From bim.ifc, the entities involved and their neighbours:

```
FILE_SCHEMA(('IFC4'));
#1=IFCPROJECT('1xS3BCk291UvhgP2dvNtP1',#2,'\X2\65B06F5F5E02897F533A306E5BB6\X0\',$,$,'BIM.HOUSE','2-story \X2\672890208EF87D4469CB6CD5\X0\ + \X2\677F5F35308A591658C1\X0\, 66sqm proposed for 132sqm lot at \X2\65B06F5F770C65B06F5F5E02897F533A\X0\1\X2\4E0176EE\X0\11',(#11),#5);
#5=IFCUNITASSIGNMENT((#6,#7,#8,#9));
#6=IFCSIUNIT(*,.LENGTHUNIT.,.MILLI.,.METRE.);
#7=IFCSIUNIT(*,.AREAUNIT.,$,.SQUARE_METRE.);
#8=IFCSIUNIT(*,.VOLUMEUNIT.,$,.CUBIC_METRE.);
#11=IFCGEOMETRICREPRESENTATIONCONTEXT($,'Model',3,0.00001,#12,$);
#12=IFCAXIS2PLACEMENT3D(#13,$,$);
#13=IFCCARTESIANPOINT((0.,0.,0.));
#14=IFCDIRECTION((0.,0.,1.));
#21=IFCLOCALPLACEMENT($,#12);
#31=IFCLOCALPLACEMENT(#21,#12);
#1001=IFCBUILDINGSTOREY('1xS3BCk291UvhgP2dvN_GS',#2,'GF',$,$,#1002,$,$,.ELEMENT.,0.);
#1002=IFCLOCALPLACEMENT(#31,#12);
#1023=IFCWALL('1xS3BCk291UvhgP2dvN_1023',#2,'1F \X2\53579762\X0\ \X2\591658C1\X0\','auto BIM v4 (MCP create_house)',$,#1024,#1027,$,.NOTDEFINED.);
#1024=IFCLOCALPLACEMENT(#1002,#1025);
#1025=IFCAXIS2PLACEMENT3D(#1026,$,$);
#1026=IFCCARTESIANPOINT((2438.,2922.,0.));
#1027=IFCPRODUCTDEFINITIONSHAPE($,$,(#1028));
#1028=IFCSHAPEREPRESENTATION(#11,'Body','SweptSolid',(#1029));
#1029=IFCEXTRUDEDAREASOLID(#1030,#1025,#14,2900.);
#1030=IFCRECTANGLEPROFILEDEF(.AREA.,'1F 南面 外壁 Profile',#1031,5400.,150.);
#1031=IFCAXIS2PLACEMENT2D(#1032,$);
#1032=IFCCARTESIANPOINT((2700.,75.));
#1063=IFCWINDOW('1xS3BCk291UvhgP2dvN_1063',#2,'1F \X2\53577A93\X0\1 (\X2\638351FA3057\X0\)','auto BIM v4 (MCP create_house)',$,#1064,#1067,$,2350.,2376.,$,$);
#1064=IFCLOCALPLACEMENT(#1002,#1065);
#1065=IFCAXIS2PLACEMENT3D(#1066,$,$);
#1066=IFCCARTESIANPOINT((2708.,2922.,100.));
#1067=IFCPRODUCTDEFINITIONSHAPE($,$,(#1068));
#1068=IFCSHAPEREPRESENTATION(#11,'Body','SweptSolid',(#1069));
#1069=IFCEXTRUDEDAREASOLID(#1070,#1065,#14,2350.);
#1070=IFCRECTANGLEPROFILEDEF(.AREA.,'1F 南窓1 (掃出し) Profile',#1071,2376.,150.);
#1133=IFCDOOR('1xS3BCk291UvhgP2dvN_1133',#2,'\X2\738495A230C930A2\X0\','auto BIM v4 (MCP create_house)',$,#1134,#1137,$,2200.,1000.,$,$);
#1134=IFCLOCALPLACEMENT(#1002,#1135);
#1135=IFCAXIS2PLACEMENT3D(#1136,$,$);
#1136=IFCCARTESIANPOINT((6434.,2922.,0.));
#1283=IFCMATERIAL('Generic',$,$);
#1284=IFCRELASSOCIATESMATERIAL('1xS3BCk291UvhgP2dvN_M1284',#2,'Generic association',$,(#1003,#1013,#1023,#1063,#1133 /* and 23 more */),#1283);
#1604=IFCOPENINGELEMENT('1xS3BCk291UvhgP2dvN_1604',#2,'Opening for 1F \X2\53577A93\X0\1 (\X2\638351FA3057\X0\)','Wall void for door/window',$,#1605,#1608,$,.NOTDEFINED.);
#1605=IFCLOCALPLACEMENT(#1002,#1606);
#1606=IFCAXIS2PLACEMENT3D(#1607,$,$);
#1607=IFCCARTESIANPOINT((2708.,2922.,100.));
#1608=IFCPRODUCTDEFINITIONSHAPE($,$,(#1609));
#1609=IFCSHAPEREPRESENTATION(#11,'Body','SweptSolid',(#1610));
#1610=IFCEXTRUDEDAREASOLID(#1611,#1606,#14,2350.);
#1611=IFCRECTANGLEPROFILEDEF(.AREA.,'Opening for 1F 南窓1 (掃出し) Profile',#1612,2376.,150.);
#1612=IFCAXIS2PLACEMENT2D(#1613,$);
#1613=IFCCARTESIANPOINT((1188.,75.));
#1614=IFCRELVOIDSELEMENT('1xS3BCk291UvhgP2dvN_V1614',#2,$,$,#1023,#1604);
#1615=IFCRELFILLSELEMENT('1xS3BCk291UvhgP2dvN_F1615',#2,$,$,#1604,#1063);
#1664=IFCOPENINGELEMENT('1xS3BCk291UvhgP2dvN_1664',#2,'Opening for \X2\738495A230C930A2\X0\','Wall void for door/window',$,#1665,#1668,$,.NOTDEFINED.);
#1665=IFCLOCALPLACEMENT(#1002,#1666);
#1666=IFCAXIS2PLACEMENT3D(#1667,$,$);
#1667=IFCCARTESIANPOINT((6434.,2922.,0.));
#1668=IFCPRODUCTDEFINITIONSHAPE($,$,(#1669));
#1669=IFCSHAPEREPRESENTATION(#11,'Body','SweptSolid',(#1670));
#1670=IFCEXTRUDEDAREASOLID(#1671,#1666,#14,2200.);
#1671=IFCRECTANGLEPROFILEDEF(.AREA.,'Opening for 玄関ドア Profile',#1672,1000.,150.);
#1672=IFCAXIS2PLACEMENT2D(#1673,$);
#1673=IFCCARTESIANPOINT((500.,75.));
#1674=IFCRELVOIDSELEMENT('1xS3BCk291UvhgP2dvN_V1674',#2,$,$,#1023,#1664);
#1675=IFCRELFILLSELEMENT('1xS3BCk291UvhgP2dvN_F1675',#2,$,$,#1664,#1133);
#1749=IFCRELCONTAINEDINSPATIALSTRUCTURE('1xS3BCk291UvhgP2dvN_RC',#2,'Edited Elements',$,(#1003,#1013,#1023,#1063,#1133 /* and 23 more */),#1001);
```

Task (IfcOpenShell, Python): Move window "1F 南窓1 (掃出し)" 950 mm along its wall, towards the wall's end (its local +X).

```python
import ifcopenshell
import ifcopenshell.api.geometry
import ifcopenshell.util.placement
import ifcopenshell.util.unit

model = ifcopenshell.open("bim.ifc")
unit_scale = ifcopenshell.util.unit.calculate_unit_scale(model)

window = model.by_guid("1xS3BCk291UvhgP2dvN_1063")
opening = window.FillsVoids[0].RelatingOpeningElement
wall = opening.VoidsElements[0].RelatingBuildingElement

wall_matrix = ifcopenshell.util.placement.get_local_placement(wall.ObjectPlacement)
shift = wall_matrix[:3, 0] * 0.95 / unit_scale
before = ifcopenshell.util.placement.get_local_placement(window.ObjectPlacement)[:3, 3].copy()

# The window is not placed relative to its opening, so move both.
for product in (opening, window):
    matrix = ifcopenshell.util.placement.get_local_placement(product.ObjectPlacement)
    matrix[:3, 3] += shift
    ifcopenshell.api.geometry.edit_object_placement(model, product=product, matrix=matrix, is_si=False)

after = ifcopenshell.util.placement.get_local_placement(window.ObjectPlacement)[:3, 3]
print("window moved by", (after - before).round(3) + 0.0)

model.write("bim-out.ifc")
```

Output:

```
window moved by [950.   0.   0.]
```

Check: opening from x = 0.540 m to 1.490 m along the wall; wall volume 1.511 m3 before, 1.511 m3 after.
